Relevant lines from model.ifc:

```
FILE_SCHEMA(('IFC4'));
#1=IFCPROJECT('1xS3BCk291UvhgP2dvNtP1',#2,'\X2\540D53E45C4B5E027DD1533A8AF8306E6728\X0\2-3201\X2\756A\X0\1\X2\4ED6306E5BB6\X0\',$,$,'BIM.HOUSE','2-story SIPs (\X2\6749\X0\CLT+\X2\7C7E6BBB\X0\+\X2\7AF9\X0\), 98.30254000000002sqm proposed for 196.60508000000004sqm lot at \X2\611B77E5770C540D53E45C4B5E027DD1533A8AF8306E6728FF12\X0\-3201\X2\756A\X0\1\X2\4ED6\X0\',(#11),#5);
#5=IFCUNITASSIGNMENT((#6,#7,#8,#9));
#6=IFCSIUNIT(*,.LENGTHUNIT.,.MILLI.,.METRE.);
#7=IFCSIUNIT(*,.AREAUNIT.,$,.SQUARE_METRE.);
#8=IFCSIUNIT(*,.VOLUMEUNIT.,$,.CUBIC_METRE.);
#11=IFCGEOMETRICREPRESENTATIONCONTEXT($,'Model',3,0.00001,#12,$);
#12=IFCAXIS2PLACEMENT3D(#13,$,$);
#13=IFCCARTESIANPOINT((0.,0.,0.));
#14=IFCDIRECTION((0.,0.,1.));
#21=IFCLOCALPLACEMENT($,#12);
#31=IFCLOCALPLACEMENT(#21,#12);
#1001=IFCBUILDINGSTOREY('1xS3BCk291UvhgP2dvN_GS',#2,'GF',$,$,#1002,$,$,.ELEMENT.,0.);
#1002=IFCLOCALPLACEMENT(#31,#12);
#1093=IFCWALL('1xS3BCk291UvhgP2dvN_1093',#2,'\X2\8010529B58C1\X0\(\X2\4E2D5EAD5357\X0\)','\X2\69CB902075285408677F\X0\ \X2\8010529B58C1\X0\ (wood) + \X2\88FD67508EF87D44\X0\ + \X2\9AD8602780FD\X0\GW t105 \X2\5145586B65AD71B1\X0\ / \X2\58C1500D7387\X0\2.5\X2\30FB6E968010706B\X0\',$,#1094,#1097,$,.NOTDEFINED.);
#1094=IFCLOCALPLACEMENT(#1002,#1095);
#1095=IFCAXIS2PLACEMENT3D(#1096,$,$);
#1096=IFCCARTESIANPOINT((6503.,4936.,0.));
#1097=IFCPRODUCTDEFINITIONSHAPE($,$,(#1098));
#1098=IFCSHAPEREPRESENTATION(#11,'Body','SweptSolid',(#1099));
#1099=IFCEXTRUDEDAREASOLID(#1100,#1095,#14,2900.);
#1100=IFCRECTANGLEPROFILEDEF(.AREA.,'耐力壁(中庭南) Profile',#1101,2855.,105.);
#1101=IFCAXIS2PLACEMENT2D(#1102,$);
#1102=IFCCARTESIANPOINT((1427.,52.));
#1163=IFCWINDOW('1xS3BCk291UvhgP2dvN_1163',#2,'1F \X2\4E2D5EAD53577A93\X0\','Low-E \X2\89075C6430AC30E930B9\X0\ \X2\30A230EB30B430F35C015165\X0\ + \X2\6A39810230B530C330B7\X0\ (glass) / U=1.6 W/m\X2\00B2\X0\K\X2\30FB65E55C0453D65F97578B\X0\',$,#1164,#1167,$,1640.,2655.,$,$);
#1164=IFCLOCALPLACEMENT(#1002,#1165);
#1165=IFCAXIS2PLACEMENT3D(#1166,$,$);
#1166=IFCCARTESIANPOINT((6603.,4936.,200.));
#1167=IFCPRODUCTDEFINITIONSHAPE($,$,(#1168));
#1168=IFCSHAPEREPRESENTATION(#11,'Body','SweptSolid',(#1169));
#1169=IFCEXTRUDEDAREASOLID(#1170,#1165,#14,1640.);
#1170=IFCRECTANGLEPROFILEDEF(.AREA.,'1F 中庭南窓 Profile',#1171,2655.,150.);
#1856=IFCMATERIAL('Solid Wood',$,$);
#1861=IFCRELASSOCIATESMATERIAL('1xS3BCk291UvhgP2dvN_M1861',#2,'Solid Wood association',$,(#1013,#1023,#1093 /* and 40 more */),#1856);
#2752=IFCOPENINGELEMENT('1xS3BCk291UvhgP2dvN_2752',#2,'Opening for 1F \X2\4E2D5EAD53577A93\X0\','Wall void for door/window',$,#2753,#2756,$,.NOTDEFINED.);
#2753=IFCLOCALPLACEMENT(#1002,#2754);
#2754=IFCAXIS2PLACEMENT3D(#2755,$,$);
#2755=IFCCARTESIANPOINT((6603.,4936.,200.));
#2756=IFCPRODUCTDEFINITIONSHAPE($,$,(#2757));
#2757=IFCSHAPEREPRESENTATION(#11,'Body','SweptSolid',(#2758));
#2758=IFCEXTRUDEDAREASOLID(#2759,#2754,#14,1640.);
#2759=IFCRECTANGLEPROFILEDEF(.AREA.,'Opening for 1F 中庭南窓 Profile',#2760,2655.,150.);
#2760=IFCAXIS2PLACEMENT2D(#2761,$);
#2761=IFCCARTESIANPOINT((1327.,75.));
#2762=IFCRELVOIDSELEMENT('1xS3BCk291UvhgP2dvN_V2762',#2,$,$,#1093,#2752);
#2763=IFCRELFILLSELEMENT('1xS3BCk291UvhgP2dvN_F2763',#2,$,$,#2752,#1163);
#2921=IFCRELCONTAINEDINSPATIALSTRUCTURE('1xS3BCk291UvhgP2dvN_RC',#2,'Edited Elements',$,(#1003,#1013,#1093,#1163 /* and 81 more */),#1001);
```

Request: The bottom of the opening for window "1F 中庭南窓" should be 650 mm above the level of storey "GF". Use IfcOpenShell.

```python
import numpy as np
import ifcopenshell
import ifcopenshell.api.geometry
import ifcopenshell.geom
import ifcopenshell.util.element
import ifcopenshell.util.placement
import ifcopenshell.util.shape
import ifcopenshell.util.unit

model = ifcopenshell.open("model.ifc")
unit_scale = ifcopenshell.util.unit.calculate_unit_scale(model)

window = model.by_id(1163)
opening = window.FillsVoids[0].RelatingOpeningElement
storey = ifcopenshell.util.element.get_container(window, ifc_class="IfcBuildingStorey")
level = ifcopenshell.util.placement.get_local_placement(storey.ObjectPlacement)[2, 3]

# The opening's origin need not be at the sill, so measure its lowest point.
shape = ifcopenshell.geom.create_shape(ifcopenshell.geom.settings(), opening)
bottom = ifcopenshell.util.shape.get_shape_bottom_elevation(shape, shape.geometry) / unit_scale
dz = level + 0.65 / unit_scale - bottom

shift = np.array([0.0, 0.0, dz])
# The window is not placed relative to its opening, so move both.
for product in (opening, window):
    matrix = ifcopenshell.util.placement.get_local_placement(product.ObjectPlacement)
    matrix[:3, 3] += shift
    ifcopenshell.api.geometry.edit_object_placement(model, product=product, matrix=matrix, is_si=False)

print(f"moved by {dz * unit_scale:+.3f} m")

model.write("model_edited.ifc")
```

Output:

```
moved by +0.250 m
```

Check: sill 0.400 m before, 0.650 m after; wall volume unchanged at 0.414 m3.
